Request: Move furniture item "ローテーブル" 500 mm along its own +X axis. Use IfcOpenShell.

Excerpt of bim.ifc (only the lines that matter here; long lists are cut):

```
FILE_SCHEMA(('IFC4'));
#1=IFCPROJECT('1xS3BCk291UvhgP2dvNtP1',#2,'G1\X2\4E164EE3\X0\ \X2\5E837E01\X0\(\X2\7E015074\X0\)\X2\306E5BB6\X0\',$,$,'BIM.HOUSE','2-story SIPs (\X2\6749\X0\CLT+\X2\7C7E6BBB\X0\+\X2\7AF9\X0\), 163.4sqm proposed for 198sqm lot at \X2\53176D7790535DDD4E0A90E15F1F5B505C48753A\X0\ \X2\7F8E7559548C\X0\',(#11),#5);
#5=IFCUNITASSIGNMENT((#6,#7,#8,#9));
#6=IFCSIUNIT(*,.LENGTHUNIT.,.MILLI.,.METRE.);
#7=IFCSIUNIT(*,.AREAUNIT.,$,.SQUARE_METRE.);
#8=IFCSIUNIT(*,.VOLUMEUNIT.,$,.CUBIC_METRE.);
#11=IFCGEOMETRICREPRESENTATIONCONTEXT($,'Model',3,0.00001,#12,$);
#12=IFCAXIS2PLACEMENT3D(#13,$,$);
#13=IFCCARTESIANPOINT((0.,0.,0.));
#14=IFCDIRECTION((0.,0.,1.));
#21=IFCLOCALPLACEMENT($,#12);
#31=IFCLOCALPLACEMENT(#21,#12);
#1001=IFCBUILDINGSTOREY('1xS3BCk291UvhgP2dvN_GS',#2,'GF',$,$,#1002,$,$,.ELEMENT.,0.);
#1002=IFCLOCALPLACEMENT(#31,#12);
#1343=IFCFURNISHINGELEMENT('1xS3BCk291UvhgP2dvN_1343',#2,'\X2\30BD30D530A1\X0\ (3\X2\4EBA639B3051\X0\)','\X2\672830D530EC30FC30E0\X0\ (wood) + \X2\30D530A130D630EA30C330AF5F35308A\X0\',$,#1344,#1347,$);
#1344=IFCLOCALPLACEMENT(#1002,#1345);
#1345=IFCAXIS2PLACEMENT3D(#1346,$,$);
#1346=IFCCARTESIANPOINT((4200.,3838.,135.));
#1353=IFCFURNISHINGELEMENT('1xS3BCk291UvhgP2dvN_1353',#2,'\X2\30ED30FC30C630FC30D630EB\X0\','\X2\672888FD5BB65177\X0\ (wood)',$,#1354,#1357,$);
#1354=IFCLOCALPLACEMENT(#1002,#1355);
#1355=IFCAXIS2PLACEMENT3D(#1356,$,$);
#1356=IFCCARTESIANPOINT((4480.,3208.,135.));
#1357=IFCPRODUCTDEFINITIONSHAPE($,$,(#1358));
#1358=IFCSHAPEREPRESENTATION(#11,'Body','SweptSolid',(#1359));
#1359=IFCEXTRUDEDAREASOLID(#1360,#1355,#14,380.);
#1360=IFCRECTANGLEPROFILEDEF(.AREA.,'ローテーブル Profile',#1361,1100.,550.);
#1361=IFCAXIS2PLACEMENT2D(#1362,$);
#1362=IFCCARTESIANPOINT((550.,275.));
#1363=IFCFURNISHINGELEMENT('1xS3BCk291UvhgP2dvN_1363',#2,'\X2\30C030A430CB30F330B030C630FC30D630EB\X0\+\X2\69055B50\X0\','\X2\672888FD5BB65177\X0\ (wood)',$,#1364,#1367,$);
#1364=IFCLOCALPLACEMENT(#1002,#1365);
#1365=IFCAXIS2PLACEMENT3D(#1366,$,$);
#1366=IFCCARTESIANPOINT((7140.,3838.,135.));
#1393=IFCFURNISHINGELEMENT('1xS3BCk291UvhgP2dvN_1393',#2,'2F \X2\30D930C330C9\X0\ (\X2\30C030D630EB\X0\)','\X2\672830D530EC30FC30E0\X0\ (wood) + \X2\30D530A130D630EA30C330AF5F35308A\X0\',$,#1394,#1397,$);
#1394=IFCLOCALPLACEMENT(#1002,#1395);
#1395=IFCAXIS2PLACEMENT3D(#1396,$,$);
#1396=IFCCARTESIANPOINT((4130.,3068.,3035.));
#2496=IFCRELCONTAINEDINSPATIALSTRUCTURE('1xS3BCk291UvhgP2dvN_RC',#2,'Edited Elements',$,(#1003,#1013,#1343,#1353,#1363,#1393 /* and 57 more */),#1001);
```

```python
import ifcopenshell
import ifcopenshell.api.geometry
import ifcopenshell.util.placement

model = ifcopenshell.open("bim.ifc")

item = model.by_id(1353)
matrix = ifcopenshell.util.placement.get_local_placement(item.ObjectPlacement)
matrix[:3, 3] += matrix[:3, 0] * 500.0
ifcopenshell.api.geometry.edit_object_placement(model, product=item, matrix=matrix, is_si=False)

print(ifcopenshell.util.placement.get_local_placement(item.ObjectPlacement).round(3) + 0.0)

model.write("bim_updated.ifc")
```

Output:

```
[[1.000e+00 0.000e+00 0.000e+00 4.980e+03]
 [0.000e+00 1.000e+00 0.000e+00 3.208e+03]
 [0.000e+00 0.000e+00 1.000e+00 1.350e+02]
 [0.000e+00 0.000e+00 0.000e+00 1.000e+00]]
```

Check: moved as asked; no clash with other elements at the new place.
